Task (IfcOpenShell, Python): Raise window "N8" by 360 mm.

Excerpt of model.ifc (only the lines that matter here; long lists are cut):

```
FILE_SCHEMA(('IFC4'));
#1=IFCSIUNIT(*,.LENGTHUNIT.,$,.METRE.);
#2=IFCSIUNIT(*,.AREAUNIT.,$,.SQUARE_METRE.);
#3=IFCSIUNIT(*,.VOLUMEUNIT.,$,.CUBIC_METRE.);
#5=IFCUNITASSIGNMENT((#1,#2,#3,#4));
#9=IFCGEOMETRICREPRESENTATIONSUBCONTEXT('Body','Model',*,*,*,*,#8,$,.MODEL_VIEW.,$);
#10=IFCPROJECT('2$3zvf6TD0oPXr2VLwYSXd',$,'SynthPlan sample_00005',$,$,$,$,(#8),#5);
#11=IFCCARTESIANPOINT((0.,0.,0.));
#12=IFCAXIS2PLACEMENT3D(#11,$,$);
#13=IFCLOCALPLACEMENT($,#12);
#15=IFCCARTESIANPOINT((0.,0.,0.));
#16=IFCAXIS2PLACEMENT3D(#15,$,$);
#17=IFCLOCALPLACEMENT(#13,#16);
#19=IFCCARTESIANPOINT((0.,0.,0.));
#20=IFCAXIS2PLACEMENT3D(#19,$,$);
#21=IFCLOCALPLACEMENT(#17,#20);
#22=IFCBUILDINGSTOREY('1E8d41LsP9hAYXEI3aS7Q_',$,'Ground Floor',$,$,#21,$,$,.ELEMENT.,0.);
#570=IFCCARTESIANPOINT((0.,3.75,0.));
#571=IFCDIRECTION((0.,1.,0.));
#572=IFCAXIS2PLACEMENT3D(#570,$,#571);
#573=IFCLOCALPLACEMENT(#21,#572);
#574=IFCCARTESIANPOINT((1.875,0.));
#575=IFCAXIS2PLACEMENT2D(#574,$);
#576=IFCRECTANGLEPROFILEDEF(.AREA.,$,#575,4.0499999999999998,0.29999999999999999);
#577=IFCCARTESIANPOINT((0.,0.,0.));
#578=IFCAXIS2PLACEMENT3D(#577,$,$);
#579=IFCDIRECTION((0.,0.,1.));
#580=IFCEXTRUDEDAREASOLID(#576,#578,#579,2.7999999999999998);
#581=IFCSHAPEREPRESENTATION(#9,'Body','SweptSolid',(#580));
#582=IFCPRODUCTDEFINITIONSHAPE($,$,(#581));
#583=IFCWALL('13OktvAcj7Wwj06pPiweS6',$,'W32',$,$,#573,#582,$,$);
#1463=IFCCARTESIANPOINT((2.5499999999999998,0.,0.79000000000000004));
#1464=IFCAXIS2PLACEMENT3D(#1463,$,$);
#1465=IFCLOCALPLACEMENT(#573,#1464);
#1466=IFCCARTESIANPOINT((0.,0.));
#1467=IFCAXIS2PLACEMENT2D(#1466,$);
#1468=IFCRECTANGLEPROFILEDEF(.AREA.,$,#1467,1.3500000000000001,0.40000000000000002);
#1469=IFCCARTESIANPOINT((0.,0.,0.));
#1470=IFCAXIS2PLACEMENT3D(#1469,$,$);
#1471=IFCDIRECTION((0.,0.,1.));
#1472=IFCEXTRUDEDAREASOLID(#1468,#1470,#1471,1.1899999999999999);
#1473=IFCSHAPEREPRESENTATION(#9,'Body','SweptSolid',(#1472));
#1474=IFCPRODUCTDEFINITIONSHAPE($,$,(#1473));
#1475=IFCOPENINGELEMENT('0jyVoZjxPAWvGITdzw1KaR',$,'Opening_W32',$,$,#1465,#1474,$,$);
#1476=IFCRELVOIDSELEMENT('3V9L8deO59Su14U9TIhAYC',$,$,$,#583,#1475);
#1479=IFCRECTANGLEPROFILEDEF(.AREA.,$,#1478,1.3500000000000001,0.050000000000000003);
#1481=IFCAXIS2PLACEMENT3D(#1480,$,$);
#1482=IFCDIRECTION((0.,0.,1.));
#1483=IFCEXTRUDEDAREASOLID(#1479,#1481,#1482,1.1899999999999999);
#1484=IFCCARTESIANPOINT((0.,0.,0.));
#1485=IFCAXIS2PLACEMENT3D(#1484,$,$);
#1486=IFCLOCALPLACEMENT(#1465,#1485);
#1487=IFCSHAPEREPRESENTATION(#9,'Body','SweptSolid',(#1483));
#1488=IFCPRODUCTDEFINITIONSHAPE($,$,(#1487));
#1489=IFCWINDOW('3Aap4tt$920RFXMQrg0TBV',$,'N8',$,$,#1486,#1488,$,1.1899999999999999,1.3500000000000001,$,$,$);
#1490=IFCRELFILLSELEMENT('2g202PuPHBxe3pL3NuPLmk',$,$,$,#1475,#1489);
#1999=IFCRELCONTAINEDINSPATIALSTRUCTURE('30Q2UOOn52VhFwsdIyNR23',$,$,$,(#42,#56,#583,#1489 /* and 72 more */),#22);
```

```python
import numpy as np
import ifcopenshell
import ifcopenshell.api.geometry
import ifcopenshell.util.placement
import ifcopenshell.util.unit

model = ifcopenshell.open("model.ifc")
unit_scale = ifcopenshell.util.unit.calculate_unit_scale(model)

window = model.by_id(1489)
opening = window.FillsVoids[0].RelatingOpeningElement
dz = 0.36 / unit_scale

shift = np.array([0.0, 0.0, dz])
# The window is placed relative to its opening, so it follows when the opening moves.
matrix = ifcopenshell.util.placement.get_local_placement(opening.ObjectPlacement)
matrix[:3, 3] += shift
ifcopenshell.api.geometry.edit_object_placement(
    model, product=opening, matrix=matrix, is_si=False, should_transform_children=True
)

print(f"moved by {dz * unit_scale:+.3f} m")

model.write("model_v2.ifc")
```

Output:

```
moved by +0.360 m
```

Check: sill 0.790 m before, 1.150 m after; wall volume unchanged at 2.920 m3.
